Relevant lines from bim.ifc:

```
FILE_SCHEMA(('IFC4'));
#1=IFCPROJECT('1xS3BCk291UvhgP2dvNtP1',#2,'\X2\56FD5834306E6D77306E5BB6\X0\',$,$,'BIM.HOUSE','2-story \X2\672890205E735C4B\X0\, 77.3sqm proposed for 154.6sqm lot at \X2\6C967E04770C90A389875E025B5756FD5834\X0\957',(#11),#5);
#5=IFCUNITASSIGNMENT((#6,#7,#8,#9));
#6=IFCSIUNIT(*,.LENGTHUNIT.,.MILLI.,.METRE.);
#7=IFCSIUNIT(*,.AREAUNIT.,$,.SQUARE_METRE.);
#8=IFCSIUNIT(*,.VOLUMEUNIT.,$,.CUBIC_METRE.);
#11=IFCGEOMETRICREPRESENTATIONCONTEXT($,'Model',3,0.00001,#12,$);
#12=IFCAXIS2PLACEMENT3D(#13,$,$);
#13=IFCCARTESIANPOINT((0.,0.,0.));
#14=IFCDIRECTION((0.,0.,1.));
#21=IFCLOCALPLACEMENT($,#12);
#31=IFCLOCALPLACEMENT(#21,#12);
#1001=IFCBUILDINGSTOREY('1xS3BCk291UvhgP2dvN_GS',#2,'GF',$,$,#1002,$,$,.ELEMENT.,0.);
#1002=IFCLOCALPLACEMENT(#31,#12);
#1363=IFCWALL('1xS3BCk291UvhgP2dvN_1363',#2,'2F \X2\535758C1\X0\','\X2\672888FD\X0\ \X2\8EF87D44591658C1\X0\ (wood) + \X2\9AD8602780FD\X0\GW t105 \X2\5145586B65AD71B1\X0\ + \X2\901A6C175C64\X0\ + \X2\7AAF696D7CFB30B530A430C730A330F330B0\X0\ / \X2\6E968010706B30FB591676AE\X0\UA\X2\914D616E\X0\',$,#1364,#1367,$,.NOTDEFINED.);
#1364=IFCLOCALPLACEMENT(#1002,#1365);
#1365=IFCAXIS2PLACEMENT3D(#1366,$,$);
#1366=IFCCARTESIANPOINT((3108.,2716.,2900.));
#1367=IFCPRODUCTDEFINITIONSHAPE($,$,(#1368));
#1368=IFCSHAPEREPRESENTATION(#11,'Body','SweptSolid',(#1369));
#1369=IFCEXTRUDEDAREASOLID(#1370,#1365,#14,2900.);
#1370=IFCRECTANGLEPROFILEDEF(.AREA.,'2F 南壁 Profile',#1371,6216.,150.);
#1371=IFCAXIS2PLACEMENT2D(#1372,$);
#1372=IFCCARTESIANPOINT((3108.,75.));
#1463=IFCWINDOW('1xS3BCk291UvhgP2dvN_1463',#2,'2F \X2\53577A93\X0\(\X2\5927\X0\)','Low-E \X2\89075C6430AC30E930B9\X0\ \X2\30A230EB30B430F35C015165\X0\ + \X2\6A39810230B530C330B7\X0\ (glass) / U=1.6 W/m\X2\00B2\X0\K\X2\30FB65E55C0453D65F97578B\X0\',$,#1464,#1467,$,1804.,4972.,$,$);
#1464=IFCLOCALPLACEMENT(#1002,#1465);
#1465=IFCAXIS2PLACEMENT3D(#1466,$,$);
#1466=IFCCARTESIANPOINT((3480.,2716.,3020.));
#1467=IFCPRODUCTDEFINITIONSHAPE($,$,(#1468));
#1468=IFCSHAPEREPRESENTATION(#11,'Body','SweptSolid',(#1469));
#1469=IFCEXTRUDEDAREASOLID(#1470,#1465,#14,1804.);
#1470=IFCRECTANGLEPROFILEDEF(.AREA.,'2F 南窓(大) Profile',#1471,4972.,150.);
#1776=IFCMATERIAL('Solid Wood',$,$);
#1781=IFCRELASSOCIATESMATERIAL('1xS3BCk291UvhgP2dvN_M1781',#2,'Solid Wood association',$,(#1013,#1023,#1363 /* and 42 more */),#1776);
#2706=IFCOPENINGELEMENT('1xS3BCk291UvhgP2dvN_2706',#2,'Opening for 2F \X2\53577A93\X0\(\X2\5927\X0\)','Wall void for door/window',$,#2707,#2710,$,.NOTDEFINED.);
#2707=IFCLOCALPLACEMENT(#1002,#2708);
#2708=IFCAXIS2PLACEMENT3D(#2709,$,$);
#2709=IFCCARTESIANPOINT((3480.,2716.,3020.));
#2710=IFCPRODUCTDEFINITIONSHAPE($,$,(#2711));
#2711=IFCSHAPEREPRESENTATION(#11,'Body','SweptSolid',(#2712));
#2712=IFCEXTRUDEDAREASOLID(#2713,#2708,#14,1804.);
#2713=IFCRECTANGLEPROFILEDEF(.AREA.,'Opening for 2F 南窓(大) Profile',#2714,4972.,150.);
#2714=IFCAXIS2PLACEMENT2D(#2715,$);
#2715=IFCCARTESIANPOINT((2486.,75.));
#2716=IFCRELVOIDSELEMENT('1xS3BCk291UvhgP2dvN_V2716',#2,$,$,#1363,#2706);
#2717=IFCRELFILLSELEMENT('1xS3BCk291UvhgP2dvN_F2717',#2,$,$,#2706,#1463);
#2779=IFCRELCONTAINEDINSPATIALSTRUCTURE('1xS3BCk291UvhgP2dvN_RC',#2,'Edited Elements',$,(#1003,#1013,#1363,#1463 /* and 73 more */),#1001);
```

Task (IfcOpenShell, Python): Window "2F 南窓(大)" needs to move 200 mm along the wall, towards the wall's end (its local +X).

```python
import ifcopenshell
import ifcopenshell.api.geometry
import ifcopenshell.util.placement

model = ifcopenshell.open("bim.ifc")

window = model.by_id(1463)
opening = window.FillsVoids[0].RelatingOpeningElement
wall = opening.VoidsElements[0].RelatingBuildingElement

wall_matrix = ifcopenshell.util.placement.get_local_placement(wall.ObjectPlacement)
shift = wall_matrix[:3, 0] * 200.0
before = ifcopenshell.util.placement.get_local_placement(window.ObjectPlacement)[:3, 3].copy()

# The window is not placed relative to its opening, so move both.
for product in (opening, window):
    matrix = ifcopenshell.util.placement.get_local_placement(product.ObjectPlacement)
    matrix[:3, 3] += shift
    ifcopenshell.api.geometry.edit_object_placement(model, product=product, matrix=matrix, is_si=False)

after = ifcopenshell.util.placement.get_local_placement(window.ObjectPlacement)[:3, 3]
print("window moved by", (after - before).round(3) + 0.0)

model.write("bim-out.ifc")
```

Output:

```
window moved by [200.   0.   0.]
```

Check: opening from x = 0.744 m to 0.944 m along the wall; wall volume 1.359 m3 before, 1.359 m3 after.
